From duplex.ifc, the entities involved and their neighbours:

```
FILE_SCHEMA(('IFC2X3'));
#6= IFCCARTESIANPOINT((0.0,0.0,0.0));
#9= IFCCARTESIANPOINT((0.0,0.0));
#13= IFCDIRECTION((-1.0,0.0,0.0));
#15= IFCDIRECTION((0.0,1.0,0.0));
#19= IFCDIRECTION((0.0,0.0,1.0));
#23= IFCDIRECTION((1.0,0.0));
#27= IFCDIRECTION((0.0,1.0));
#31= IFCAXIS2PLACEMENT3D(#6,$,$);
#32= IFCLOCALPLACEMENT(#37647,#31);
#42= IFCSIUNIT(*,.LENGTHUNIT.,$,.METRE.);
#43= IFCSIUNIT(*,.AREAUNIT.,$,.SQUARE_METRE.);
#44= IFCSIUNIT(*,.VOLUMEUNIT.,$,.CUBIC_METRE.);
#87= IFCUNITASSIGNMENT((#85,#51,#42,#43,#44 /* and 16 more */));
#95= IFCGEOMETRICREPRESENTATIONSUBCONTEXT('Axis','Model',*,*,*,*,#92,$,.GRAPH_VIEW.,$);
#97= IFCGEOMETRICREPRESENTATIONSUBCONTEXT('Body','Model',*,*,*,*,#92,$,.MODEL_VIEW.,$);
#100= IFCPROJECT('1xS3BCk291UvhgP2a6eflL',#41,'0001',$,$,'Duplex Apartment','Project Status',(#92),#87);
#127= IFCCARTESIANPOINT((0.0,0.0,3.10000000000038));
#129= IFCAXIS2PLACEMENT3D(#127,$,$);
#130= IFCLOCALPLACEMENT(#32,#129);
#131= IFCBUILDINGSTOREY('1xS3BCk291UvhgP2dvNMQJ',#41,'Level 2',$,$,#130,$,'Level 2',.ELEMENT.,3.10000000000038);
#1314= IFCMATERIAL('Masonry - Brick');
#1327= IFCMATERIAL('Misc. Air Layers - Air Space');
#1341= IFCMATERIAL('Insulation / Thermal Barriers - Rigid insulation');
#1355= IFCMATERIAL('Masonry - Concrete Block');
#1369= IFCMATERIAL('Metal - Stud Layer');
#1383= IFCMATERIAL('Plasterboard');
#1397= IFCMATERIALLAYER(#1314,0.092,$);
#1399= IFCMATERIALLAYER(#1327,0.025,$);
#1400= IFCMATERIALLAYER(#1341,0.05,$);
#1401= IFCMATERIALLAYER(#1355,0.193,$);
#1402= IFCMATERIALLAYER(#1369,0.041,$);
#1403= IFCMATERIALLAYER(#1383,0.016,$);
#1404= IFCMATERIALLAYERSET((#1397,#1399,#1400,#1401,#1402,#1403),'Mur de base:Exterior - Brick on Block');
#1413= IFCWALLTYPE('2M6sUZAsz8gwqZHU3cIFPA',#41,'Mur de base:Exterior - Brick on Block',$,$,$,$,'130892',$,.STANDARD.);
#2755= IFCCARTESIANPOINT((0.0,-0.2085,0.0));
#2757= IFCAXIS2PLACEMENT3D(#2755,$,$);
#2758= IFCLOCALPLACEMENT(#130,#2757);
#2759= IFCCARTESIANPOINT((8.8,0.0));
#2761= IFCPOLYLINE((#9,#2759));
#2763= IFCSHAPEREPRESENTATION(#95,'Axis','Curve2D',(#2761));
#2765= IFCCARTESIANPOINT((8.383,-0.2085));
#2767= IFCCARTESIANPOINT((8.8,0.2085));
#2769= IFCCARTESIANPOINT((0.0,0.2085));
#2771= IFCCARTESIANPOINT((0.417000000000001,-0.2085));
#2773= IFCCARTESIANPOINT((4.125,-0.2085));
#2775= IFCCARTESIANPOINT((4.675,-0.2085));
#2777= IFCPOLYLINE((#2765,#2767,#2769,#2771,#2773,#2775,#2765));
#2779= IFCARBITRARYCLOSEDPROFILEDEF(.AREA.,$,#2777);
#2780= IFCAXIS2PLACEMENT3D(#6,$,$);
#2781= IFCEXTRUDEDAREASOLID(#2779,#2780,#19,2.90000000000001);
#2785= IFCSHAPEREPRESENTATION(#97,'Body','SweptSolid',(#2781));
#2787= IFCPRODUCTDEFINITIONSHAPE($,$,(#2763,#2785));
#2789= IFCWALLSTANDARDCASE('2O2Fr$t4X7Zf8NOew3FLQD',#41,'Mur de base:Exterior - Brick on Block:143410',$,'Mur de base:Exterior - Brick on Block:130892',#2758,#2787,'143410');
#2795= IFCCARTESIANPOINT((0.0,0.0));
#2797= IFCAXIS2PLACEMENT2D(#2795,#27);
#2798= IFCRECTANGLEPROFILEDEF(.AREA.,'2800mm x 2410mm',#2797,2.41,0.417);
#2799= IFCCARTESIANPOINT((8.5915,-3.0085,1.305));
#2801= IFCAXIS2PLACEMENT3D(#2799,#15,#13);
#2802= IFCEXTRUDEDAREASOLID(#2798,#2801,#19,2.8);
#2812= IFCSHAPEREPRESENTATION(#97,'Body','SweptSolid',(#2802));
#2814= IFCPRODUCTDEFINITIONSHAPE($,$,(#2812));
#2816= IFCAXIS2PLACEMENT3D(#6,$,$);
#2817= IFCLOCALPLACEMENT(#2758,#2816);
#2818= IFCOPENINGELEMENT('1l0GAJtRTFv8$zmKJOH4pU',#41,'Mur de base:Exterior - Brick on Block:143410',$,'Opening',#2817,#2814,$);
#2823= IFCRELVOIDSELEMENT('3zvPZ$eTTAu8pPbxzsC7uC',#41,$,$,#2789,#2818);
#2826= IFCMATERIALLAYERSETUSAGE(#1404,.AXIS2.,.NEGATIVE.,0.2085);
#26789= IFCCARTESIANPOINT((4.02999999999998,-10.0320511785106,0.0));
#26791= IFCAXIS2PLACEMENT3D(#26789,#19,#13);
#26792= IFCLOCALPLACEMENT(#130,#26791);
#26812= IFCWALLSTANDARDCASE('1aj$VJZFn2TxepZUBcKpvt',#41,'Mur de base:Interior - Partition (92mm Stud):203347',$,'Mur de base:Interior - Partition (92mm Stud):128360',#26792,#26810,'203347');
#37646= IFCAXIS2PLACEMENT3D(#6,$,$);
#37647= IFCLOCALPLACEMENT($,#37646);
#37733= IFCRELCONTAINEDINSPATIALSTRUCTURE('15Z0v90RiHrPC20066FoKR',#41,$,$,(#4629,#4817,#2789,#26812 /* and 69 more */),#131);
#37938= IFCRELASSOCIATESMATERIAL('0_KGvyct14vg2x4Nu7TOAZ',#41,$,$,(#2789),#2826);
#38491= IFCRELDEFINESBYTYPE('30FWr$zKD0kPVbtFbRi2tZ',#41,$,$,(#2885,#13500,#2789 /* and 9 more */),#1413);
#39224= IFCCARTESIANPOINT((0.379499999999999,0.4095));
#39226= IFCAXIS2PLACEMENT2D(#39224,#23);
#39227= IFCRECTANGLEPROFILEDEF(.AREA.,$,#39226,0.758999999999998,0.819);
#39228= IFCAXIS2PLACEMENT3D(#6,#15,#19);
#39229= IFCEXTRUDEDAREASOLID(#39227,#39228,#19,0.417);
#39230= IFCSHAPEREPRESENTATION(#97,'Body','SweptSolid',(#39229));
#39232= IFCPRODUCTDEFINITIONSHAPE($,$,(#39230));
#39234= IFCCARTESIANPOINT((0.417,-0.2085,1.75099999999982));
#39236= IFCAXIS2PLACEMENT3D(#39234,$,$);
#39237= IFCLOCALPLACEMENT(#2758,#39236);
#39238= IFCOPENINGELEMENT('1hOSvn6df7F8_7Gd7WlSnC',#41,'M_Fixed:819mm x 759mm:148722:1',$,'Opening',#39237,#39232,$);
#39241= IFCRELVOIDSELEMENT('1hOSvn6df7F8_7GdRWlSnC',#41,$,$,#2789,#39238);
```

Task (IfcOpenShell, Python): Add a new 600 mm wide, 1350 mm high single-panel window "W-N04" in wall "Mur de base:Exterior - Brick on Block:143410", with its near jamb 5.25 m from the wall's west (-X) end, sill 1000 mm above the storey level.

```python
import numpy as np
import ifcopenshell
import ifcopenshell.api.feature
import ifcopenshell.api.geometry
import ifcopenshell.api.root
import ifcopenshell.api.spatial
import ifcopenshell.api.type
import ifcopenshell.geom
import ifcopenshell.util.element
import ifcopenshell.util.placement
import ifcopenshell.util.representation
import ifcopenshell.util.shape
import ifcopenshell.util.unit

model = ifcopenshell.open("duplex.ifc")
unit_scale = ifcopenshell.util.unit.calculate_unit_scale(model)
settings = ifcopenshell.geom.settings()


def volume(element):
    """Net volume in cubic metres, openings subtracted."""
    shape = ifcopenshell.geom.create_shape(settings, element)
    return ifcopenshell.util.shape.get_volume(shape.geometry)


wall = model.by_guid("2O2Fr$t4X7Zf8NOew3FLQD")
storey = ifcopenshell.util.element.get_container(wall, ifc_class="IfcBuildingStorey")
context = ifcopenshell.util.representation.get_context(model, "Model", "Body", "MODEL_VIEW")
before = volume(wall)

width, height, from_end, sill = 0.6, 1.35, 5.25, 1  # metres

# The wall runs along its own X axis, and the end named is its -X end.
wall_shape = ifcopenshell.geom.create_shape(settings, wall)
x, y, z = ifcopenshell.util.shape.get_vertices(wall_shape.geometry).T
start = x.min() + from_end
face, thickness = float(y.min()), float(y.max() - y.min())
wall_matrix = ifcopenshell.util.placement.get_local_placement(wall.ObjectPlacement)
level = ifcopenshell.util.placement.get_local_placement(storey.ObjectPlacement)[2, 3]


def in_wall(x, y):
    """Placement at x, y metres in the wall's axes, at sill height."""
    matrix = wall_matrix.copy()
    matrix[:, 3] = wall_matrix @ np.array([x / unit_scale, y / unit_scale, 0.0, 1.0])
    matrix[2, 3] = level + sill / unit_scale
    return matrix


# Opening: a box that overshoots both wall faces by 50 mm.
opening = ifcopenshell.api.root.create_entity(model, ifc_class="IfcOpeningElement")
box = ifcopenshell.api.geometry.add_wall_representation(
    model, context=context, length=width, height=height, thickness=thickness + 0.1
)
ifcopenshell.api.geometry.assign_representation(model, product=opening, representation=box)
ifcopenshell.api.geometry.edit_object_placement(model, product=opening, matrix=in_wall(start, face - 0.05), is_si=False)
ifcopenshell.api.feature.add_feature(model, feature=opening, element=wall)

window = ifcopenshell.api.root.create_entity(model, ifc_class="IfcWindow", name="W-N04")
window.OverallWidth, window.OverallHeight = width / unit_scale, height / unit_scale
body = ifcopenshell.api.geometry.add_window_representation(
    model,
    context=context,
    overall_width=window.OverallWidth,
    overall_height=window.OverallHeight,
    partition_type="SINGLE_PANEL",
)
ifcopenshell.api.geometry.assign_representation(model, product=window, representation=body)
ifcopenshell.api.spatial.assign_container(model, products=[window], relating_structure=storey)
fills = ifcopenshell.api.feature.add_filling(model, opening=opening, element=window)
fills.OwnerHistory = window.OwnerHistory  # required in IFC2X3

# IFC2X3 keeps the operation on the window style.
style = ifcopenshell.api.root.create_entity(model, ifc_class="IfcWindowStyle", name="W-N04")
style.OperationType, style.ConstructionType = "SINGLE_PANEL", "NOTDEFINED"
style.ParameterTakesPrecedence = style.Sizeable = False
ifcopenshell.api.type.assign_type(model, related_objects=[window], relating_type=style)

# Centre the window in the wall's thickness.
ifcopenshell.api.geometry.edit_object_placement(model, product=window, matrix=in_wall(start, face), is_si=False)
window_shape = ifcopenshell.geom.create_shape(settings, window)
depth = ifcopenshell.util.shape.get_vertices(window_shape.geometry)[:, 1]
offset = face + thickness / 2 - (depth.min() + depth.max()) / 2
ifcopenshell.api.geometry.edit_object_placement(model, product=window, matrix=in_wall(start, offset), is_si=False)

after = volume(wall)

print(f"wall volume {before:.3f} -> {after:.3f} m3")

model.write("duplex_updated.ifc")
```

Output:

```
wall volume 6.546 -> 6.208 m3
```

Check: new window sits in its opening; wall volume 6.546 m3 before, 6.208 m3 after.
